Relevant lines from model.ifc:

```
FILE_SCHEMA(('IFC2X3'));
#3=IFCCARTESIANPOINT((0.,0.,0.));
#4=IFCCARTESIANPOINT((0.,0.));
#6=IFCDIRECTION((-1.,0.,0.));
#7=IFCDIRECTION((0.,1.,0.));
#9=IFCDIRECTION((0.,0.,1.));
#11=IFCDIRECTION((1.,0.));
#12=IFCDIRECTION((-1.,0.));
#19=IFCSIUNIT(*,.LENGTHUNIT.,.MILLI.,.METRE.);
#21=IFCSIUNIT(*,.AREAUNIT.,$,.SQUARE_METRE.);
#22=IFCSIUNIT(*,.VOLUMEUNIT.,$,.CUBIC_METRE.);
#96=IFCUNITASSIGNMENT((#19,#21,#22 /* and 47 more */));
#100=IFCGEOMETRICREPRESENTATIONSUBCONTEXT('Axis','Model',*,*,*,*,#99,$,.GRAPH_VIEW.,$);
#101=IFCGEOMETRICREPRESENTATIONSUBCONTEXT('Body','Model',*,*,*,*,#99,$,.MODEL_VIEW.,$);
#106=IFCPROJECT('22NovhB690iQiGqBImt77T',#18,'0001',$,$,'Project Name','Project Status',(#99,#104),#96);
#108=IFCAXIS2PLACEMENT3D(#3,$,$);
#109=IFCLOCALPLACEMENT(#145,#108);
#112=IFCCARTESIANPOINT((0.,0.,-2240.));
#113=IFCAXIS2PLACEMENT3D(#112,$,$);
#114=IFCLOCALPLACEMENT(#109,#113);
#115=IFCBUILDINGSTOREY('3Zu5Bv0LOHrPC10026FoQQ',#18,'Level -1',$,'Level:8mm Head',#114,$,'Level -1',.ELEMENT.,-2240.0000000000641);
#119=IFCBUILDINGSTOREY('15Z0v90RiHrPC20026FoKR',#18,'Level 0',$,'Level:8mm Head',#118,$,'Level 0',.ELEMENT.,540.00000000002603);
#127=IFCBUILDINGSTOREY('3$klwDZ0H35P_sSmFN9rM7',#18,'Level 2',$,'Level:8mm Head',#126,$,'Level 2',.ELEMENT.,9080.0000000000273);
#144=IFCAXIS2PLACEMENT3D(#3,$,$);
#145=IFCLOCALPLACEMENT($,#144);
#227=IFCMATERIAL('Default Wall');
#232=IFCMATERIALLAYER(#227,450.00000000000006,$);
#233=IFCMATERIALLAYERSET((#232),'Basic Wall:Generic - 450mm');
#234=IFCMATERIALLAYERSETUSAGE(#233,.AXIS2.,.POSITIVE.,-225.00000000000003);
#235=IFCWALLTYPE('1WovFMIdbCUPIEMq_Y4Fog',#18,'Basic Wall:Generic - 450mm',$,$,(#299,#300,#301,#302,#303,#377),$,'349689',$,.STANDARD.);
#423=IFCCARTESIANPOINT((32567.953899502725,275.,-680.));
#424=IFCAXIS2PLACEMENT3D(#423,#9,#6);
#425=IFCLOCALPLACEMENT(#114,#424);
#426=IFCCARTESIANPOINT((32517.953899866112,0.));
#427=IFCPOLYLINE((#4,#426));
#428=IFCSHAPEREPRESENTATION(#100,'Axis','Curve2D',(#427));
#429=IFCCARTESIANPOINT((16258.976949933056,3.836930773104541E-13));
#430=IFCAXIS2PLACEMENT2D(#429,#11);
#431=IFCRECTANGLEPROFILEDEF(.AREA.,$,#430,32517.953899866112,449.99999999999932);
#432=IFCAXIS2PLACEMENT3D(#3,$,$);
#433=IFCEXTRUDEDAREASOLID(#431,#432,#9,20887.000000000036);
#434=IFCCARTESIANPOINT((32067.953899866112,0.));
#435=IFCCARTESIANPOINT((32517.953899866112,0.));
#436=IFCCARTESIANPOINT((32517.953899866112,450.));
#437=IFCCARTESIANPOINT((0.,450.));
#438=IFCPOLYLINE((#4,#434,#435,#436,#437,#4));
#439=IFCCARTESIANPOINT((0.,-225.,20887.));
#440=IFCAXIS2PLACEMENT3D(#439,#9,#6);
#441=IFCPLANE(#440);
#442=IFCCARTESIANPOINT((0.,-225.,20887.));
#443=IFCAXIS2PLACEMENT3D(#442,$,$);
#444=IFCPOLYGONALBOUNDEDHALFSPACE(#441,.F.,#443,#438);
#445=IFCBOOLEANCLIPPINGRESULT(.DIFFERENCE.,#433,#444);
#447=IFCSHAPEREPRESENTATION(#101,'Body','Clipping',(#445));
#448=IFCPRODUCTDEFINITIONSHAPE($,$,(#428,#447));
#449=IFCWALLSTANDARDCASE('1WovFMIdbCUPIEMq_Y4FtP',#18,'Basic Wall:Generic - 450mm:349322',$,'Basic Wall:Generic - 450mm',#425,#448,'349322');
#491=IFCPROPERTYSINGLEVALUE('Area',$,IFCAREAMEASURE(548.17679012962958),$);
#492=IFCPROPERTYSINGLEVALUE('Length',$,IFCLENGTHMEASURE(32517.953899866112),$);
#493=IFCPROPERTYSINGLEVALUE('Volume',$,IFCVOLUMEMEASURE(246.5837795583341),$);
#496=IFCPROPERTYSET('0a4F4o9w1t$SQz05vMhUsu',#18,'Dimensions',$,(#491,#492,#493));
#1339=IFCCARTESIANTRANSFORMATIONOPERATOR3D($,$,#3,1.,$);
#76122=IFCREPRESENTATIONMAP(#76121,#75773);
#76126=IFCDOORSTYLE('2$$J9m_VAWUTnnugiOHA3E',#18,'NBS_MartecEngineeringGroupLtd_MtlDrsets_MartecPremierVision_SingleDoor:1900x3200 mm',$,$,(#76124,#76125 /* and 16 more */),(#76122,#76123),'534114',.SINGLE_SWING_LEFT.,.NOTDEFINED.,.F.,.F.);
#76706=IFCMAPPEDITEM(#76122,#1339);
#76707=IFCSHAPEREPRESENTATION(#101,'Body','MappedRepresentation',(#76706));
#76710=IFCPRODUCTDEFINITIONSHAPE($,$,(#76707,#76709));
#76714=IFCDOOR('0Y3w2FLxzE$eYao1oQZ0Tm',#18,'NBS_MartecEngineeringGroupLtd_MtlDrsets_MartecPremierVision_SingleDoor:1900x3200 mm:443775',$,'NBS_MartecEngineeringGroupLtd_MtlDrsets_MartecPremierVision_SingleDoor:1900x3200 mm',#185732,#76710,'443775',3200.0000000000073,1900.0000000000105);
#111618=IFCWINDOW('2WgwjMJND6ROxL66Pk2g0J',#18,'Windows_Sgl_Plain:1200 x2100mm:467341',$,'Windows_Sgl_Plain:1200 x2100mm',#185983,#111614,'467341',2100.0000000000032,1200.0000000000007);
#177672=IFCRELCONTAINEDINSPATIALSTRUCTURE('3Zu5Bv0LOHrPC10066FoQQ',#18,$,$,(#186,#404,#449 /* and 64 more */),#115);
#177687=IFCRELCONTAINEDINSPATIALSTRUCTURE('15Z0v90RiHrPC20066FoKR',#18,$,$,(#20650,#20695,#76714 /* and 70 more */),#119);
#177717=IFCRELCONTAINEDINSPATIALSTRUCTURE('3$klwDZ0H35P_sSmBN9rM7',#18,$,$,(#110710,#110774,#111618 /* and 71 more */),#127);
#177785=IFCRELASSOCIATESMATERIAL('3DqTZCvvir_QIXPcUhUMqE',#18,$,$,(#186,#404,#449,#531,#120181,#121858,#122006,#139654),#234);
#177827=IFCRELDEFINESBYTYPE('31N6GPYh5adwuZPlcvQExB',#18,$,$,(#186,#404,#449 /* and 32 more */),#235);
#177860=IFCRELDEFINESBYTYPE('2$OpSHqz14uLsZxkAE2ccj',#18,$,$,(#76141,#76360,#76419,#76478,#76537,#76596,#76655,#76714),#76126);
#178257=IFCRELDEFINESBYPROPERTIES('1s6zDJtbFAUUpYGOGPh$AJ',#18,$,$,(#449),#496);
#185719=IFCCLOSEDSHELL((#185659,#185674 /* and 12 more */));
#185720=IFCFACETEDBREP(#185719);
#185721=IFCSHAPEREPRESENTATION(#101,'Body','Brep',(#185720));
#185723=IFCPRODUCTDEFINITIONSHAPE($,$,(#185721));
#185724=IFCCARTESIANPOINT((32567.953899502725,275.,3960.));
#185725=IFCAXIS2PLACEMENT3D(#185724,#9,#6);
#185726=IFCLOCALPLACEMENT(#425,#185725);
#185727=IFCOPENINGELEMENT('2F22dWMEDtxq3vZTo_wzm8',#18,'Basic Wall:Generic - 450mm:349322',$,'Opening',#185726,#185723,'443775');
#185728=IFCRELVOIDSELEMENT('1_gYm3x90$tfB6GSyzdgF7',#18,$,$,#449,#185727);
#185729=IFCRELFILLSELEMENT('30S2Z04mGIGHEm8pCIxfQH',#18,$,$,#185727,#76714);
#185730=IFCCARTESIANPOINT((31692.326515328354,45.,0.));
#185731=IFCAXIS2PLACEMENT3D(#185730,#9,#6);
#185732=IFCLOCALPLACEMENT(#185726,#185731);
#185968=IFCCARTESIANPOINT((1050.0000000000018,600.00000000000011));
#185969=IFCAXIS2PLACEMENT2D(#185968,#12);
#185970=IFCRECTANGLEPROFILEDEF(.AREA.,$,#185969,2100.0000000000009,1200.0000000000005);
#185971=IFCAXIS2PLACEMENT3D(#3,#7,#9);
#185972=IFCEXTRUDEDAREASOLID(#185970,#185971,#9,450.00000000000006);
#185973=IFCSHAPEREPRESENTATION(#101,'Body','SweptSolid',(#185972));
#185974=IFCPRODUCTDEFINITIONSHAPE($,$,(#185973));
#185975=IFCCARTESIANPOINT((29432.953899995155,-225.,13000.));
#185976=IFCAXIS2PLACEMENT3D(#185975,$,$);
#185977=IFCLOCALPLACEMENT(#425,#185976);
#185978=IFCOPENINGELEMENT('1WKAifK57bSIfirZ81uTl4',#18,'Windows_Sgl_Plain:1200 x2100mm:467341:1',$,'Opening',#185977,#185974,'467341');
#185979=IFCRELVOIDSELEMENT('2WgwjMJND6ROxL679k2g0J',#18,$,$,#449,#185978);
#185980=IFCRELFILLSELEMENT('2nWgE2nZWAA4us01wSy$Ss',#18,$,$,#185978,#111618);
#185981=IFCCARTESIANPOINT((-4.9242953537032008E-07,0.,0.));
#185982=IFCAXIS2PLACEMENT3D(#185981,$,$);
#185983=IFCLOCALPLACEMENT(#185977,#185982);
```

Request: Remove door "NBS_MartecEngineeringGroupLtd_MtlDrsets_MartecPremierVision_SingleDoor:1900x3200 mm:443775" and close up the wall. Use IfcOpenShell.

```python
import ifcopenshell
import ifcopenshell.api.feature
import ifcopenshell.api.pset
import ifcopenshell.api.root
import ifcopenshell.geom
import ifcopenshell.util.element
import ifcopenshell.util.shape
import ifcopenshell.util.unit

model = ifcopenshell.open("model.ifc")
area_scale = ifcopenshell.util.unit.calculate_unit_scale(model, "AREAUNIT")
volume_scale = ifcopenshell.util.unit.calculate_unit_scale(model, "VOLUMEUNIT")
settings = ifcopenshell.geom.settings()


def volume(element):
    """Net volume in cubic metres, openings subtracted."""
    shape = ifcopenshell.geom.create_shape(settings, element)
    return ifcopenshell.util.shape.get_volume(shape.geometry)


door = model.by_guid("0Y3w2FLxzE$eYao1oQZ0Tm")
opening = door.FillsVoids[0].RelatingOpeningElement
wall = opening.VoidsElements[0].RelatingBuildingElement
before = volume(wall)

ifcopenshell.api.root.remove_product(model, product=door)
ifcopenshell.api.feature.remove_feature(model, feature=opening)

after = volume(wall)
thickness = 0.45  # wall thickness in metres

# Update the wall's stored quantities.
pset = model.by_id(ifcopenshell.util.element.get_pset(wall, "Dimensions", should_inherit=False)["id"])
ifcopenshell.api.pset.edit_pset(model, pset=pset, properties={
    "Area": model.create_entity("IfcAreaMeasure", after / thickness / area_scale),
    "Volume": model.create_entity("IfcVolumeMeasure", after / volume_scale),
})

print(f"wall volume {before:.3f} -> {after:.3f} m3")

model.write("model-out.ifc")
```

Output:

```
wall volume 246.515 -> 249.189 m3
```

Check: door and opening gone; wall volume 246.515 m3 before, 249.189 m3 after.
